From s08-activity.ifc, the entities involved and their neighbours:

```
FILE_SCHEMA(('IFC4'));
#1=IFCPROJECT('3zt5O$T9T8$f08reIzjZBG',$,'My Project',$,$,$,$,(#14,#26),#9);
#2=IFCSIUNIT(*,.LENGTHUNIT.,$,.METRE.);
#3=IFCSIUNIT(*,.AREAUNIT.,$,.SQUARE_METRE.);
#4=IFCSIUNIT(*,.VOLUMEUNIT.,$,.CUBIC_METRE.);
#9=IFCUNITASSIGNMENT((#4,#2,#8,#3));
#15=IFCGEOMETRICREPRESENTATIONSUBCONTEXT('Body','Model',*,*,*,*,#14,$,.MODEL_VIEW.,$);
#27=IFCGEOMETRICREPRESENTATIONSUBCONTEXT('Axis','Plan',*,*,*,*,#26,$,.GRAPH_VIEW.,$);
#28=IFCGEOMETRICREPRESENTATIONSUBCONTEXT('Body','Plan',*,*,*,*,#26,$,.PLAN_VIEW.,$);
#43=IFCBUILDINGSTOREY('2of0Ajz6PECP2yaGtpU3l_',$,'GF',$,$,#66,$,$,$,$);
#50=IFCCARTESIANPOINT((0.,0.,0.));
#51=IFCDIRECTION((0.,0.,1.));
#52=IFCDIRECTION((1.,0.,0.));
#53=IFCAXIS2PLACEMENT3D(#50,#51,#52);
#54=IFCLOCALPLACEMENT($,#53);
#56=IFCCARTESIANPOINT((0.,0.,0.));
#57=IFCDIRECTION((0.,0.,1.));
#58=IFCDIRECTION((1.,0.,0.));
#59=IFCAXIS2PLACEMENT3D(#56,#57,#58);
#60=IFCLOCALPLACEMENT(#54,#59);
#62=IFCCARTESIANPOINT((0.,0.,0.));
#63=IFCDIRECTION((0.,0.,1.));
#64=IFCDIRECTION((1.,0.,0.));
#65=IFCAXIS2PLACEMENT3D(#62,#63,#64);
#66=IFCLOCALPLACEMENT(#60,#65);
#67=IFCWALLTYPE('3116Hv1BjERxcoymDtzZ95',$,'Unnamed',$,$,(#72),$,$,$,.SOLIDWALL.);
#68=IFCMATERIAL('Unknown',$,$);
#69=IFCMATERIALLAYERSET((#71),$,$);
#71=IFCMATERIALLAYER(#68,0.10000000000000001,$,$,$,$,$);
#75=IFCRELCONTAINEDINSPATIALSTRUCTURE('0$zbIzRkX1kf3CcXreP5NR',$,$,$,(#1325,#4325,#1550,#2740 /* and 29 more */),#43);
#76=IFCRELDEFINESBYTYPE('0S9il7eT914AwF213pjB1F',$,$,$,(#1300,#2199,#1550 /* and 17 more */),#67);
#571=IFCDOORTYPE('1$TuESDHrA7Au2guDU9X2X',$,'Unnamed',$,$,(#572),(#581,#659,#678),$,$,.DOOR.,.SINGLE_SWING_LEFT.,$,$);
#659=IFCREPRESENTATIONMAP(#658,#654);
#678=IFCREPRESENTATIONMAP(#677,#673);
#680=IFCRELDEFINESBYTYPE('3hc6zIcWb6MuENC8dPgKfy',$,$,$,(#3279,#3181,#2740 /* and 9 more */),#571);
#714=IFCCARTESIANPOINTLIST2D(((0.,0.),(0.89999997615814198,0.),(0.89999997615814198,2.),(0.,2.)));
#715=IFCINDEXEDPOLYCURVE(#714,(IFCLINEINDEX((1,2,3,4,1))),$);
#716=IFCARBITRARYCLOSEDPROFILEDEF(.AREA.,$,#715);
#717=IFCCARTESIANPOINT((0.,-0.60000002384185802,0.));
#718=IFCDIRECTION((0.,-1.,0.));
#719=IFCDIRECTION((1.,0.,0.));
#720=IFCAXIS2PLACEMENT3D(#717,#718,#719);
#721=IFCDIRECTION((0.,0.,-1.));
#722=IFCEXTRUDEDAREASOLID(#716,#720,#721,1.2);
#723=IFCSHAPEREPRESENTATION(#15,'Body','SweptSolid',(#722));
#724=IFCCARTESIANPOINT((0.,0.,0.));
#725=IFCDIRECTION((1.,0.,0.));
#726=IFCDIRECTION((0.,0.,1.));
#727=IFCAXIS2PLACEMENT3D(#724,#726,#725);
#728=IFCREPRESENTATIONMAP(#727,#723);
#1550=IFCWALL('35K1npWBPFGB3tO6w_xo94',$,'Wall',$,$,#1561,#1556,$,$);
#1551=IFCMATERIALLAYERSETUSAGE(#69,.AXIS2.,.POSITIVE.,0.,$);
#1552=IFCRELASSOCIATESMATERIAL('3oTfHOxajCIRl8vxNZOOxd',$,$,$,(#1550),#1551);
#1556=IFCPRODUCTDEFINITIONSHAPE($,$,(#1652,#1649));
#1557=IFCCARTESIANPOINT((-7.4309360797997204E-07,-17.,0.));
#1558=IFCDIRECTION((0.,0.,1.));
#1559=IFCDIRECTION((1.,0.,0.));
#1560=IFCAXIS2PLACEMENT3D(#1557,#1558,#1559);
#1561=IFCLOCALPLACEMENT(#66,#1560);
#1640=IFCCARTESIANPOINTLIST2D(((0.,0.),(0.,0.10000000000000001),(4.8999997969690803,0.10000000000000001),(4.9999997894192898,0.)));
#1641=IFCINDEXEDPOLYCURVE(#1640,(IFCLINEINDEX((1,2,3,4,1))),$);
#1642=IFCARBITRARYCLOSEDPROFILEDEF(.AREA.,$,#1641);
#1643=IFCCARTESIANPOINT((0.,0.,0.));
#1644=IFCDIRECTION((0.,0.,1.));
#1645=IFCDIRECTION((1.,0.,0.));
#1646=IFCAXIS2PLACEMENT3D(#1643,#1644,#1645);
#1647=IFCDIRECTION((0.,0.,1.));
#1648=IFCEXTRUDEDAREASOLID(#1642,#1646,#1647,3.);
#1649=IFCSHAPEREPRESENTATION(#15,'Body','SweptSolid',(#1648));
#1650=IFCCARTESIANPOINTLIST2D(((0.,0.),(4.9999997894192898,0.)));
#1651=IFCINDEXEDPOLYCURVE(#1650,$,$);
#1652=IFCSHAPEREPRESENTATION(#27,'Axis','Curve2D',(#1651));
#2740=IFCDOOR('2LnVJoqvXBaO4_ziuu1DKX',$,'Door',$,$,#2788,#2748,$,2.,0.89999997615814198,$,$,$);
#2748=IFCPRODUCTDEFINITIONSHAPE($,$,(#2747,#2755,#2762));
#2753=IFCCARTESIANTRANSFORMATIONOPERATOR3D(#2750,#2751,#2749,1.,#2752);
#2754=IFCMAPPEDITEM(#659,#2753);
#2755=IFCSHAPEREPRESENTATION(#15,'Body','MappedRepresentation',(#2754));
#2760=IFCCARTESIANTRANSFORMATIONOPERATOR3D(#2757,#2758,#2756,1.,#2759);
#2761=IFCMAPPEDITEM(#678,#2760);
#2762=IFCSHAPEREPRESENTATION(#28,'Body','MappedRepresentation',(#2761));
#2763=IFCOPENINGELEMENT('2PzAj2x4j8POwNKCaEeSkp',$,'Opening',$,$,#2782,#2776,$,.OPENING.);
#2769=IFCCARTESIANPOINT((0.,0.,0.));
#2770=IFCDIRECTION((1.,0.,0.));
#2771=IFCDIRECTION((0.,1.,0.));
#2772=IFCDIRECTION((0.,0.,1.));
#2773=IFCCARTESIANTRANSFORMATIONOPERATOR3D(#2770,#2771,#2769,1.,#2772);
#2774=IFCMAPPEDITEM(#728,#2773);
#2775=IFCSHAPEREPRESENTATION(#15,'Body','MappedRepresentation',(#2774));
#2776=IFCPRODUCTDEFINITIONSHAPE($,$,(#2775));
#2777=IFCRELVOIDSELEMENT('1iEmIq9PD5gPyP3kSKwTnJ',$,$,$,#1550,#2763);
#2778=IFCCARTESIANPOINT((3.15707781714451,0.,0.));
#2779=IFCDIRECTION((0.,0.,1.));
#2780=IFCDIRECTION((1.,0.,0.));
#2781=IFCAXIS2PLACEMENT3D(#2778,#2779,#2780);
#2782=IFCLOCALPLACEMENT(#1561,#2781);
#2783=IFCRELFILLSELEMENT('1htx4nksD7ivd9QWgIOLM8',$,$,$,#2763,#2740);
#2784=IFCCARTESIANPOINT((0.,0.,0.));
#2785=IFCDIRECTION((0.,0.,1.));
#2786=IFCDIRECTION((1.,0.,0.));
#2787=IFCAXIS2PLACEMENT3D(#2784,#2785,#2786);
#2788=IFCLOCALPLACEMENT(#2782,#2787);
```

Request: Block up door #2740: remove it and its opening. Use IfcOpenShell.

```python
import ifcopenshell
import ifcopenshell.api.feature
import ifcopenshell.api.root
import ifcopenshell.geom
import ifcopenshell.util.shape

model = ifcopenshell.open("s08-activity.ifc")
settings = ifcopenshell.geom.settings()


def volume(element):
    """Net volume in cubic metres, openings subtracted."""
    shape = ifcopenshell.geom.create_shape(settings, element)
    return ifcopenshell.util.shape.get_volume(shape.geometry)


door = model.by_guid("2LnVJoqvXBaO4_ziuu1DKX")
opening = door.FillsVoids[0].RelatingOpeningElement
wall = opening.VoidsElements[0].RelatingBuildingElement
before = volume(wall)

ifcopenshell.api.root.remove_product(model, product=door)
ifcopenshell.api.feature.remove_feature(model, feature=opening)

after = volume(wall)

print(f"wall volume {before:.3f} -> {after:.3f} m3")

model.write("s08-activity_rev.ifc")
```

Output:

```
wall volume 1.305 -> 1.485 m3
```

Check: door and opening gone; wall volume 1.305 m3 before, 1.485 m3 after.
